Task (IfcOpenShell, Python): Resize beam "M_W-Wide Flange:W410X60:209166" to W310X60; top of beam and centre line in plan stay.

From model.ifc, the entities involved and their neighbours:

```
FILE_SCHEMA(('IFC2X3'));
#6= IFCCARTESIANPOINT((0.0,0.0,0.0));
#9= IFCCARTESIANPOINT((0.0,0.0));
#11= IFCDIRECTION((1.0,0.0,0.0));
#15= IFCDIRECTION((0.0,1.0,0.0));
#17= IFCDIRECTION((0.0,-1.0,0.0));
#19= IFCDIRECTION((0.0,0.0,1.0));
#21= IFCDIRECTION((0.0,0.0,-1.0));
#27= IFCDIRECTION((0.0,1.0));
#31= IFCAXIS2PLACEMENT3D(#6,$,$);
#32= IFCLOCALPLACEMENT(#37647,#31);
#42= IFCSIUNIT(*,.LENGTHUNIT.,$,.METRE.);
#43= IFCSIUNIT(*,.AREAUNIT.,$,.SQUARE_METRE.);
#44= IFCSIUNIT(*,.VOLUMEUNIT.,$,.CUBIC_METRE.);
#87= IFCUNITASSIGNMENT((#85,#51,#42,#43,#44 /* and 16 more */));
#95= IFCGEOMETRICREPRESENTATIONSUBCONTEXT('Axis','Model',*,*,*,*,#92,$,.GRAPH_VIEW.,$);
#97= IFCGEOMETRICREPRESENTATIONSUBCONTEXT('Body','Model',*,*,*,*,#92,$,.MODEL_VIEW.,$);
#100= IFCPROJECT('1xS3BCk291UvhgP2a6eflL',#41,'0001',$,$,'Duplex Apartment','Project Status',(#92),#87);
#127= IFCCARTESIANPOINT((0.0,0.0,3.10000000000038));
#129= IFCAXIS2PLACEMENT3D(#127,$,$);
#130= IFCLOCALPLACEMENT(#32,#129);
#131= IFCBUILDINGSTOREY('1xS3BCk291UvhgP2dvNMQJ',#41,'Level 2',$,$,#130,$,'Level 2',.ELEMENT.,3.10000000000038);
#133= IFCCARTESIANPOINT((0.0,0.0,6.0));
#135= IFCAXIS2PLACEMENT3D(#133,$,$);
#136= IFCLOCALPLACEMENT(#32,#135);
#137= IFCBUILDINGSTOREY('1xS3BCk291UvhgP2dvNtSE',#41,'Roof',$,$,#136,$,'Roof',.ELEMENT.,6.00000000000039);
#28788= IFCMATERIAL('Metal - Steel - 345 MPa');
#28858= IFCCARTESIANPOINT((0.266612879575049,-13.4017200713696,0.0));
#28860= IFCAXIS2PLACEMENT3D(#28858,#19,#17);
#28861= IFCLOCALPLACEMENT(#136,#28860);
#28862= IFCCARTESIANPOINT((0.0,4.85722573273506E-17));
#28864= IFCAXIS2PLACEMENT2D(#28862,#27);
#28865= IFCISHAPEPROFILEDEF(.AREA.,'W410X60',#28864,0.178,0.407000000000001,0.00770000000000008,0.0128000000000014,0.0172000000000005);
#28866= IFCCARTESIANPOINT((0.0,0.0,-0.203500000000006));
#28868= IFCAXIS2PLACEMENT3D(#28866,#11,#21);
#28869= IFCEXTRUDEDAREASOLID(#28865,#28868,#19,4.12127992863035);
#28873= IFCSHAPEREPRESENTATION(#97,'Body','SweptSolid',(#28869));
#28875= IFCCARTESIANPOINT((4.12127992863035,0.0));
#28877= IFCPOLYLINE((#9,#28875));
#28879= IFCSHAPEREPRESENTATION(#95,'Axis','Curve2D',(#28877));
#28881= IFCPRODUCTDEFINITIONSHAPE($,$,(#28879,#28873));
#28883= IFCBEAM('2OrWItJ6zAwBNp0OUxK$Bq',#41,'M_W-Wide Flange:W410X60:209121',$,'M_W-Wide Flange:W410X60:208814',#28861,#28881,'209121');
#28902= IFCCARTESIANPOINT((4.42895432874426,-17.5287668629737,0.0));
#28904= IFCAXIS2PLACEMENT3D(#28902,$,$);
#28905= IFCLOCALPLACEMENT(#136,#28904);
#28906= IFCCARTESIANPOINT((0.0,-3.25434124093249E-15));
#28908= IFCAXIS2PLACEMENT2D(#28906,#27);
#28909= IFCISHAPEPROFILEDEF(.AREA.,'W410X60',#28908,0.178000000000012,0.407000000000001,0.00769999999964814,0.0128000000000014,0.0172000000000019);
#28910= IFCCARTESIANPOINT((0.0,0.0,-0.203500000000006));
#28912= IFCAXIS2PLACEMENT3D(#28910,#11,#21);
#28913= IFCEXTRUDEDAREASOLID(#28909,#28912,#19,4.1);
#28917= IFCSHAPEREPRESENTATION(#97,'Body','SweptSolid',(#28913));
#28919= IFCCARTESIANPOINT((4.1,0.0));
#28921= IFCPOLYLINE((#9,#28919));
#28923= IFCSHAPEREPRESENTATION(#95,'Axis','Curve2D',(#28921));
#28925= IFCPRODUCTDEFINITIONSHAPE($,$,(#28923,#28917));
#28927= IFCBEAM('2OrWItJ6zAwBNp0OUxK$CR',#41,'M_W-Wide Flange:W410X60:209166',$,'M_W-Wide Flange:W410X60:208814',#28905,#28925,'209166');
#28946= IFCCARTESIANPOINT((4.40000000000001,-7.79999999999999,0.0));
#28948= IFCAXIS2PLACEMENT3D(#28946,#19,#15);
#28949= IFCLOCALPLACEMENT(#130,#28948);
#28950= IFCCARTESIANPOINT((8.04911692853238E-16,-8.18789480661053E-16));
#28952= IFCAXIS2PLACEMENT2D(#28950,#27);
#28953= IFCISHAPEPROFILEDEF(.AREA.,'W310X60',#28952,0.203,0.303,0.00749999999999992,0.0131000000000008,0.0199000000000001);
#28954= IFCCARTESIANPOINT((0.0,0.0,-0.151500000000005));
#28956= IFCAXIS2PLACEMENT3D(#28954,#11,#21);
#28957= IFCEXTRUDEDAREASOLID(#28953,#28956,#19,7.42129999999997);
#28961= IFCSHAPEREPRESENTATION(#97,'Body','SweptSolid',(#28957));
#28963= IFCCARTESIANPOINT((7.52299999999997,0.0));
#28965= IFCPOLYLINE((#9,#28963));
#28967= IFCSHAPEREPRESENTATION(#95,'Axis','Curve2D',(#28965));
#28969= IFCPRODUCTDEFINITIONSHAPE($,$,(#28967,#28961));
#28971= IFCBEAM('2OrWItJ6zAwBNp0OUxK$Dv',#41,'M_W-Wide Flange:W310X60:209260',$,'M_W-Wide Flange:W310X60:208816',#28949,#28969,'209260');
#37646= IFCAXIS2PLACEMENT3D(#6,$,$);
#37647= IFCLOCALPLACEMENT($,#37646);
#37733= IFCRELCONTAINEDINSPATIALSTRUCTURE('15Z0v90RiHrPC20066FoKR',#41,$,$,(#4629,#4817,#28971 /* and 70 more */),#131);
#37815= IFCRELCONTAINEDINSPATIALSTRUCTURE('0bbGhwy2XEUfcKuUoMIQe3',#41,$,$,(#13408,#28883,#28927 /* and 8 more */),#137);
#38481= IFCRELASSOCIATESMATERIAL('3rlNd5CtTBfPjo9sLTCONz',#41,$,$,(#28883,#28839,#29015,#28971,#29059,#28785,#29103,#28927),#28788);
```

```python
import ifcopenshell
import ifcopenshell.util.element
import ifcopenshell.util.representation

model = ifcopenshell.open("model.ifc")

member = model.by_id(28927)
source = next(p for p in model.by_type("IfcIShapeProfileDef") if p.ProfileName == "W310X60")

body = ifcopenshell.util.representation.get_representation(member, "Model", "Body")
solid = body.Items[0]
old_profile = solid.SweptArea

# Copy the section's sizes but keep this member's own profile position.
profile = ifcopenshell.util.element.copy(model, source)
# Profiles are centred, so shift by half the change in depth to hold the top.
shift = (old_profile.OverallDepth - profile.OverallDepth) / 2
x, y = old_profile.Position.Location.Coordinates
up = (-1.0, 0.0)  # upwards, in the solid's own plane
location = model.createIfcCartesianPoint((x + up[0] * shift, y + up[1] * shift))
profile.Position = model.createIfcAxis2Placement2D(location, old_profile.Position.RefDirection)
solid.SweptArea = profile
if not model.get_total_inverses(old_profile):
    ifcopenshell.util.element.remove_deep2(model, old_profile)
member.Name = member.Name.replace("W410X60", "W310X60")
member.ObjectType = member.ObjectType.replace("W410X60", "W310X60")

print(solid.SweptArea)

model.write("model_updated.ifc")
```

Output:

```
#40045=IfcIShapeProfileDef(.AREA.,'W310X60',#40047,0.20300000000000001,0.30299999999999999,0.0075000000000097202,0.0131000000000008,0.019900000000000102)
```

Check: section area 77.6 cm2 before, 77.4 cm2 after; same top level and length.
